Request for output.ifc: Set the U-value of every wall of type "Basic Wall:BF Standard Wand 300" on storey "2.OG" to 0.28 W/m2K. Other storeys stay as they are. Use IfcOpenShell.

First a look at what the model holds.

```python
import ifcopenshell
import ifcopenshell.util.element

model = ifcopenshell.open("output.ifc")
print(model.schema)
storey = next(s for s in model.by_type("IfcBuildingStorey") if s.Name == "2.OG")
walls = [e for e in ifcopenshell.util.element.get_decomposition(storey) if e.is_a("IfcWall")]
seen = {}
for e in walls:
    element_type = ifcopenshell.util.element.get_type(e)
    key = (element_type.Name if element_type != e and element_type else None, ifcopenshell.util.element.get_pset(e, "Pset_WallCommon", "ThermalTransmittance"))
    seen[key] = seen.get(key, 0) + 1
for (name, value), count in sorted(seen.items(), key=str):
    print(count, "x", name, "|", value)
```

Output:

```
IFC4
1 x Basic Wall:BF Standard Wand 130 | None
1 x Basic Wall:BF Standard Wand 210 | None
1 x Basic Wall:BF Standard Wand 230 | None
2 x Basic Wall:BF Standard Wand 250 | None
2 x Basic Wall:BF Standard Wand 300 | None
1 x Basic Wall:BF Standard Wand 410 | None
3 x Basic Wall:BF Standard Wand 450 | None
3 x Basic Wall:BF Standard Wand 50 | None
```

```python
import ifcopenshell
import ifcopenshell.api.pset
import ifcopenshell.util.element

model = ifcopenshell.open("output.ifc")

storey = next(s for s in model.by_type("IfcBuildingStorey") if s.Name == "2.OG")
walls = [e for e in ifcopenshell.util.element.get_decomposition(storey) if e.is_a("IfcWall")]

count = 0
for e in walls:
    element_type = ifcopenshell.util.element.get_type(e)
    if element_type in (None, e) or element_type.Name != "Basic Wall:BF Standard Wand 300":
        continue
    # add_pset returns the element's existing set when there is one.
    pset = ifcopenshell.api.pset.add_pset(model, product=e, name="Pset_WallCommon")
    ifcopenshell.api.pset.edit_pset(model, pset=pset, properties={"ThermalTransmittance": 0.28})
    count += 1

print(count, "walls updated")

model.write("output_updated.ifc")
```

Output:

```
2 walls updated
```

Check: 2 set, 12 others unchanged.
